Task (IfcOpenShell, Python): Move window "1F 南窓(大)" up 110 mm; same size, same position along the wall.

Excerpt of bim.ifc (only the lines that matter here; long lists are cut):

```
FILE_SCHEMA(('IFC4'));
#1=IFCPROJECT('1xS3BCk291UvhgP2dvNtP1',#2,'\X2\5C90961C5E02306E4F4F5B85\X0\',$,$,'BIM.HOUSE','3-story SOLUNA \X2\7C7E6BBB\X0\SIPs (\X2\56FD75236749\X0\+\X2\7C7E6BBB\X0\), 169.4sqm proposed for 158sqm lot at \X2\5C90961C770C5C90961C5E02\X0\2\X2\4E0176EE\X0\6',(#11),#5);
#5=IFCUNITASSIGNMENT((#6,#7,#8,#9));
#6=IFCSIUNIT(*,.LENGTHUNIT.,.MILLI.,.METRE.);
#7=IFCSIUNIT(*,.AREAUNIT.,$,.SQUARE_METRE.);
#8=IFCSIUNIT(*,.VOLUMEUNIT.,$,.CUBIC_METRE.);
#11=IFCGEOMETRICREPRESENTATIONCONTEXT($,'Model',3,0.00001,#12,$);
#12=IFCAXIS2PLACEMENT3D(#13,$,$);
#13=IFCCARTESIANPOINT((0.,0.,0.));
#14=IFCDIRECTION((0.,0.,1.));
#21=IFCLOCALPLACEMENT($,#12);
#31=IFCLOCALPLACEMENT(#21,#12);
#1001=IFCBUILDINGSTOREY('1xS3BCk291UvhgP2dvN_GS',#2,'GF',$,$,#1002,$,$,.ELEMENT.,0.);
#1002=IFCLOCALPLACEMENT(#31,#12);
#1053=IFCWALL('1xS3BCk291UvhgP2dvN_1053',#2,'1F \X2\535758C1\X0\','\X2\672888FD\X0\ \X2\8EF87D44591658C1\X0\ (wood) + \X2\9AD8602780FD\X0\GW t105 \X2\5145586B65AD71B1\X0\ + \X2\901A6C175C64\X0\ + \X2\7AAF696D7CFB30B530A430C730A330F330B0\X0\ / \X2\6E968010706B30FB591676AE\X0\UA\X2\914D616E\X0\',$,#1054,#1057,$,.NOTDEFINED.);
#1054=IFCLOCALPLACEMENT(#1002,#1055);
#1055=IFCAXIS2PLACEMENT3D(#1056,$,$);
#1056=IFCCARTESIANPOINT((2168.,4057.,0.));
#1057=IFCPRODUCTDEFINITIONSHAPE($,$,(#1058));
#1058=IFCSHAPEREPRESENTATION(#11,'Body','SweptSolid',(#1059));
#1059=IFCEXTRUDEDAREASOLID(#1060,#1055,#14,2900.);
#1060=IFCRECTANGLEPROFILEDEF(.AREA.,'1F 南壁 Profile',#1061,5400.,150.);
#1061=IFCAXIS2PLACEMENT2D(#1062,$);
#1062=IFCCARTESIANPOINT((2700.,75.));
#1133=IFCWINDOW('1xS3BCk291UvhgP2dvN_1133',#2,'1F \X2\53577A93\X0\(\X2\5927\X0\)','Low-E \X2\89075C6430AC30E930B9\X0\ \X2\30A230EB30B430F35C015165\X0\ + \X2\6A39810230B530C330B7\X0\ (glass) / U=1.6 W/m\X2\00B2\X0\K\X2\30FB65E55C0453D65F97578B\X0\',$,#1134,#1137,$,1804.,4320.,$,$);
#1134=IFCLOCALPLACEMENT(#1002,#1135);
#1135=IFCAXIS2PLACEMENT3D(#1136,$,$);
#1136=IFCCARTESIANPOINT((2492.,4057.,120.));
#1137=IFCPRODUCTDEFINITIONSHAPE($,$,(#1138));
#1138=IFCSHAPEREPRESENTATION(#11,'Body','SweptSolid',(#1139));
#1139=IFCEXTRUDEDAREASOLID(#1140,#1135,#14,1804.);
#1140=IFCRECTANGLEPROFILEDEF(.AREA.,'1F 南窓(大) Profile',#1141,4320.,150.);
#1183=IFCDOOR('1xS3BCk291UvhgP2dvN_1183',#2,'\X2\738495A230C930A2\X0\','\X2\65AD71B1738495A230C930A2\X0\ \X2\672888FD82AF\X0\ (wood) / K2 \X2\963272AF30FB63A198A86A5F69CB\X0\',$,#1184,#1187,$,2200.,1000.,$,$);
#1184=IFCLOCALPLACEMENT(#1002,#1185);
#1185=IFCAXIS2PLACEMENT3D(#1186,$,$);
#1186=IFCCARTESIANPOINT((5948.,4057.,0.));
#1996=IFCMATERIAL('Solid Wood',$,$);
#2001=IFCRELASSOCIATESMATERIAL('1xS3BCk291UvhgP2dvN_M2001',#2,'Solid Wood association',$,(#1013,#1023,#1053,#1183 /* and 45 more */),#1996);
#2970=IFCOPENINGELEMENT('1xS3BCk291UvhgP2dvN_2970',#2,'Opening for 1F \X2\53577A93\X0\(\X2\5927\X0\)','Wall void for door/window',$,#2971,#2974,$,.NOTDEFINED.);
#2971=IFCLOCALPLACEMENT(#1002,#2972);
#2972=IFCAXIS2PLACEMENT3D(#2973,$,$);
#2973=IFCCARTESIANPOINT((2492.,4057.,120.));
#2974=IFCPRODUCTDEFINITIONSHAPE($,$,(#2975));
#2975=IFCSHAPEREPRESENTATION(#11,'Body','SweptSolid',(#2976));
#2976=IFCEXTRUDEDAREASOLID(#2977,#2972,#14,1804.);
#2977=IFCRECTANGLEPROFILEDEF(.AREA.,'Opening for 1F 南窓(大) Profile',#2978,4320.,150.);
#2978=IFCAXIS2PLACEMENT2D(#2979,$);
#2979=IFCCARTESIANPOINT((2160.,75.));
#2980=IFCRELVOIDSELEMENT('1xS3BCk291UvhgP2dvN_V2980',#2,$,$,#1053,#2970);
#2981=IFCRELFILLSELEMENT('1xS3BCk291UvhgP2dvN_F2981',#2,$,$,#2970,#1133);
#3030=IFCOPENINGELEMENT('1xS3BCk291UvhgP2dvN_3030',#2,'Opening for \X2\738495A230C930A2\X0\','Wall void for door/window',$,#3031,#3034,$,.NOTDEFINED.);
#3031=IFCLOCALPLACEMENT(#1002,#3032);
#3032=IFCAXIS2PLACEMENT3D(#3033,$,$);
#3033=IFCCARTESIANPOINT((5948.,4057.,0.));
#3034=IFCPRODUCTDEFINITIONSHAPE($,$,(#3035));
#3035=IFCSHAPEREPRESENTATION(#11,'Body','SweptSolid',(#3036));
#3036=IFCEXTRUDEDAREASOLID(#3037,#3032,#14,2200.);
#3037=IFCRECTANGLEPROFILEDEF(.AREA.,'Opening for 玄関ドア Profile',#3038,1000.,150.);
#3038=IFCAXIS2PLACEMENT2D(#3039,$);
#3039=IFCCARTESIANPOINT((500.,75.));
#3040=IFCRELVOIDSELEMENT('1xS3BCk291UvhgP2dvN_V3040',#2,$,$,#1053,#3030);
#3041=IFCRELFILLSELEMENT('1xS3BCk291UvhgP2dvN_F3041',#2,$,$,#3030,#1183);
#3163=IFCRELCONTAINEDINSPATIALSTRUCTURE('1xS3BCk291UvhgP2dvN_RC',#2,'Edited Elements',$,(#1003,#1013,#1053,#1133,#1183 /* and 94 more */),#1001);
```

```python
import numpy as np
import ifcopenshell
import ifcopenshell.api.geometry
import ifcopenshell.util.placement
import ifcopenshell.util.unit

model = ifcopenshell.open("bim.ifc")
unit_scale = ifcopenshell.util.unit.calculate_unit_scale(model)

window = model.by_guid("1xS3BCk291UvhgP2dvN_1133")
opening = window.FillsVoids[0].RelatingOpeningElement
dz = 0.11 / unit_scale

shift = np.array([0.0, 0.0, dz])
# The window is not placed relative to its opening, so move both.
for product in (opening, window):
    matrix = ifcopenshell.util.placement.get_local_placement(product.ObjectPlacement)
    matrix[:3, 3] += shift
    ifcopenshell.api.geometry.edit_object_placement(model, product=product, matrix=matrix, is_si=False)

print(f"moved by {dz * unit_scale:+.3f} m")

model.write("bim_edited.ifc")
```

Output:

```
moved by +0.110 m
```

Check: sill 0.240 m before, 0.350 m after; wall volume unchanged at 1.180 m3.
